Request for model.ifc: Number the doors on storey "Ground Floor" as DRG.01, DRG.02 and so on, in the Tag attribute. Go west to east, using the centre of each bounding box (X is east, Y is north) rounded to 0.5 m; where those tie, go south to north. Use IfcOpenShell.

First a look at what the model holds.

```python
import ifcopenshell
import ifcopenshell.util.element
import ifcopenshell.util.placement

model = ifcopenshell.open("model.ifc")
print(model.schema)
storey = next(s for s in model.by_type("IfcBuildingStorey") if s.Name == "Ground Floor")
doors = [e for e in ifcopenshell.util.element.get_decomposition(storey) if e.is_a("IfcDoor")]
for e in sorted(doors, key=lambda e: e.id()):
    origin = ifcopenshell.util.placement.get_local_placement(e.ObjectPlacement)[:3, 3]
    print(e.id(), e.Tag, e.Name, origin.round(2) + 0.0, sep=" | ")
```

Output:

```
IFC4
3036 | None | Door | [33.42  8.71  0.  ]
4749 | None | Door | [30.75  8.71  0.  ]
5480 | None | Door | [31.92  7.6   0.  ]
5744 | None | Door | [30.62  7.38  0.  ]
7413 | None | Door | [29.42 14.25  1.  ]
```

```python
import ifcopenshell
import ifcopenshell.geom
import ifcopenshell.util.element
import ifcopenshell.util.shape

model = ifcopenshell.open("model.ifc")
settings = ifcopenshell.geom.settings()
settings.set("use-world-coords", True)


def centre(element):
    shape = ifcopenshell.geom.create_shape(settings, element)
    return ifcopenshell.util.shape.get_bbox_centroid(shape.geometry)


storey = next(s for s in model.by_type("IfcBuildingStorey") if s.Name == "Ground Floor")
doors = [e for e in ifcopenshell.util.element.get_decomposition(storey) if e.is_a("IfcDoor")]

# Insertion points can sit at a corner or the storey origin, so sort by the geometry (in metres).
centres = {e: centre(e) for e in doors}
doors.sort(key=lambda e: (round(centres[e][0] / 0.5), centres[e][1]))

for i, e in enumerate(doors, start=1):
    number = f"DRG.{i:02d}"
    e.Tag = number
    print(e.id(), number)

model.write("model-out.ifc")
```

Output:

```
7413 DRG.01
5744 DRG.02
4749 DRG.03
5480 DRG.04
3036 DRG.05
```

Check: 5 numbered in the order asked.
